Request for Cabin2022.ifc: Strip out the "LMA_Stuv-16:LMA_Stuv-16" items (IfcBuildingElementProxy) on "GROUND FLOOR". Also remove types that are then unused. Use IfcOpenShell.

First a look at what the model holds.

```python
import ifcopenshell
import ifcopenshell.util.element

model = ifcopenshell.open("Cabin2022.ifc")
print(model.schema)
storey = next(s for s in model.by_type("IfcBuildingStorey") if s.Name == "GROUND FLOOR")
proxies = [e for e in ifcopenshell.util.element.get_decomposition(storey) if e.is_a("IfcBuildingElementProxy")]
seen = {}
for e in proxies:
    element_type = ifcopenshell.util.element.get_type(e)
    name = element_type.Name if element_type not in (None, e) else None
    seen[name] = seen.get(name, 0) + 1
for name, count in sorted(seen.items(), key=str):
    print(count, "x", name)
```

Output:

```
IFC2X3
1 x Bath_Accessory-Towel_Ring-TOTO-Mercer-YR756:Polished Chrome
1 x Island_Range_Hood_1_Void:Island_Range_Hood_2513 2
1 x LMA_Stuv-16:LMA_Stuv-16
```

```python
import ifcopenshell
import ifcopenshell.api.root
import ifcopenshell.util.element

model = ifcopenshell.open("Cabin2022.ifc")

storey = next(s for s in model.by_type("IfcBuildingStorey") if s.Name == "GROUND FLOOR")
proxies = [e for e in ifcopenshell.util.element.get_decomposition(storey) if e.is_a("IfcBuildingElementProxy")]
targets = [e for e in proxies if (t := ifcopenshell.util.element.get_type(e)) not in (None, e) and t.Name == "LMA_Stuv-16:LMA_Stuv-16"]
types = {ifcopenshell.util.element.get_type(e) for e in targets} - {None, *targets}

for e in targets:
    ifcopenshell.api.root.remove_product(model, product=e)
print(len(targets), "removed")

unused = [t for t in types if not ifcopenshell.util.element.get_types(t)]
for t in unused:
    ifcopenshell.api.root.remove_product(model, product=t)
print(len(unused), "unused types removed")

model.write("Cabin2022_updated.ifc")
```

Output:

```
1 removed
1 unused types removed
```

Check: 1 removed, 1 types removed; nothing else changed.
